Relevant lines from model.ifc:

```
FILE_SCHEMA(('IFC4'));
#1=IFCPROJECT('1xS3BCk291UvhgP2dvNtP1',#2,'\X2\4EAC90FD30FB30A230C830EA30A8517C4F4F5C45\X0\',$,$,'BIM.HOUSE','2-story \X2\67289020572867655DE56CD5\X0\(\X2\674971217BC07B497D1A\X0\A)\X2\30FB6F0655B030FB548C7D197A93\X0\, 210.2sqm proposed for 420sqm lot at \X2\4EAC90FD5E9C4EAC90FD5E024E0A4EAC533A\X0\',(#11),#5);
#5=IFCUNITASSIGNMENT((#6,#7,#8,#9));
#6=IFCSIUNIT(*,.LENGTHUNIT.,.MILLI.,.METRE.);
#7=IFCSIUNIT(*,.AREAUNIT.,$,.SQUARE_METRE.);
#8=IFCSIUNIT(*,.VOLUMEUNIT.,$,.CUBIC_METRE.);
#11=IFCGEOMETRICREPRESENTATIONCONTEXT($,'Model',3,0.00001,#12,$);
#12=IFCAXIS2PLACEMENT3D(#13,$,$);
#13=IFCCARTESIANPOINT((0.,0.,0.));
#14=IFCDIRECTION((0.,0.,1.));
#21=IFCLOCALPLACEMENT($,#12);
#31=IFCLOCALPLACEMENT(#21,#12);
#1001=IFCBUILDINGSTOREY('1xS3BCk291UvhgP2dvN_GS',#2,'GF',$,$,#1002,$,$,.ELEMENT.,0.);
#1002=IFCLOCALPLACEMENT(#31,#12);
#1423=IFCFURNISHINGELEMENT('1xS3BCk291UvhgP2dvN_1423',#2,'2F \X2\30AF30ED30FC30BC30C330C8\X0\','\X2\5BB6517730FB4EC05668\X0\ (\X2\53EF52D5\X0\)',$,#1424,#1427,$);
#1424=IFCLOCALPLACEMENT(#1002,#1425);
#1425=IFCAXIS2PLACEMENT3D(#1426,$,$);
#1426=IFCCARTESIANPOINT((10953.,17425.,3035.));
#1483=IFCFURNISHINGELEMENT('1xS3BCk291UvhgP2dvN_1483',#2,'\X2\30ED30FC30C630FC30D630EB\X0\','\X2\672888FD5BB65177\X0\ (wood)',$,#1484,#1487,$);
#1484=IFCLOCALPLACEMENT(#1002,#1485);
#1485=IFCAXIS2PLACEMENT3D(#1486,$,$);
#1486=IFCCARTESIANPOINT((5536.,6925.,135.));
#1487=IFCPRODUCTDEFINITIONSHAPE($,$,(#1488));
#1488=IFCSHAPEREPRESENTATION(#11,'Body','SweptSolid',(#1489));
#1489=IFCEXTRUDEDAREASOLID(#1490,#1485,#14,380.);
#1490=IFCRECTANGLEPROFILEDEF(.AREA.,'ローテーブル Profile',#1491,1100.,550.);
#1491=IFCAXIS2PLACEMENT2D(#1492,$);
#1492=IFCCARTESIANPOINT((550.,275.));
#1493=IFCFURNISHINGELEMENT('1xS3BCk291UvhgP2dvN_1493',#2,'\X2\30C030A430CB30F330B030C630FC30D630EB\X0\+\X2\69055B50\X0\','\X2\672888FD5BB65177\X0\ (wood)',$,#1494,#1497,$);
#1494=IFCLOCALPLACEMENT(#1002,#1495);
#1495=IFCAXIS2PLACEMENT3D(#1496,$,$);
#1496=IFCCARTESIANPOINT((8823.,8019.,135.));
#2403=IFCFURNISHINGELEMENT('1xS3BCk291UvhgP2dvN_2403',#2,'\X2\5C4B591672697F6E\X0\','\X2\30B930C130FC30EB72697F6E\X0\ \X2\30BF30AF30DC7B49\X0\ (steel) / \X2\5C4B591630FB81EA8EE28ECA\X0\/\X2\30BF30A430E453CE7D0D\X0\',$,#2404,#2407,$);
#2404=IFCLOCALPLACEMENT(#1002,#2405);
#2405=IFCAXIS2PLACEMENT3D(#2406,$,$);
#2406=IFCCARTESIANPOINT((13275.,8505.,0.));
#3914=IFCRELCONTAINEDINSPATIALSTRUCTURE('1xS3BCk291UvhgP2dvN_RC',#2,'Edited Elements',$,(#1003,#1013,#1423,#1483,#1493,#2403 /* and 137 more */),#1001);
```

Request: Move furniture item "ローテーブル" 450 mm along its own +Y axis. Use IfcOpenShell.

```python
import ifcopenshell
import ifcopenshell.api.geometry
import ifcopenshell.util.placement
import ifcopenshell.util.unit

model = ifcopenshell.open("model.ifc")
unit_scale = ifcopenshell.util.unit.calculate_unit_scale(model)

item = model.by_id(1483)
matrix = ifcopenshell.util.placement.get_local_placement(item.ObjectPlacement)
matrix[:3, 3] += matrix[:3, 1] * 0.45 / unit_scale
ifcopenshell.api.geometry.edit_object_placement(model, product=item, matrix=matrix, is_si=False)

print(ifcopenshell.util.placement.get_local_placement(item.ObjectPlacement).round(3) + 0.0)

model.write("model_v2.ifc")
```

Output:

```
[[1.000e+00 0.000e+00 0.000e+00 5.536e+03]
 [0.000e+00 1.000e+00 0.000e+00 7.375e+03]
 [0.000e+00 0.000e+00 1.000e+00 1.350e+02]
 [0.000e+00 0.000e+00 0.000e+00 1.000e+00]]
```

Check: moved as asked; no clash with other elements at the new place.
